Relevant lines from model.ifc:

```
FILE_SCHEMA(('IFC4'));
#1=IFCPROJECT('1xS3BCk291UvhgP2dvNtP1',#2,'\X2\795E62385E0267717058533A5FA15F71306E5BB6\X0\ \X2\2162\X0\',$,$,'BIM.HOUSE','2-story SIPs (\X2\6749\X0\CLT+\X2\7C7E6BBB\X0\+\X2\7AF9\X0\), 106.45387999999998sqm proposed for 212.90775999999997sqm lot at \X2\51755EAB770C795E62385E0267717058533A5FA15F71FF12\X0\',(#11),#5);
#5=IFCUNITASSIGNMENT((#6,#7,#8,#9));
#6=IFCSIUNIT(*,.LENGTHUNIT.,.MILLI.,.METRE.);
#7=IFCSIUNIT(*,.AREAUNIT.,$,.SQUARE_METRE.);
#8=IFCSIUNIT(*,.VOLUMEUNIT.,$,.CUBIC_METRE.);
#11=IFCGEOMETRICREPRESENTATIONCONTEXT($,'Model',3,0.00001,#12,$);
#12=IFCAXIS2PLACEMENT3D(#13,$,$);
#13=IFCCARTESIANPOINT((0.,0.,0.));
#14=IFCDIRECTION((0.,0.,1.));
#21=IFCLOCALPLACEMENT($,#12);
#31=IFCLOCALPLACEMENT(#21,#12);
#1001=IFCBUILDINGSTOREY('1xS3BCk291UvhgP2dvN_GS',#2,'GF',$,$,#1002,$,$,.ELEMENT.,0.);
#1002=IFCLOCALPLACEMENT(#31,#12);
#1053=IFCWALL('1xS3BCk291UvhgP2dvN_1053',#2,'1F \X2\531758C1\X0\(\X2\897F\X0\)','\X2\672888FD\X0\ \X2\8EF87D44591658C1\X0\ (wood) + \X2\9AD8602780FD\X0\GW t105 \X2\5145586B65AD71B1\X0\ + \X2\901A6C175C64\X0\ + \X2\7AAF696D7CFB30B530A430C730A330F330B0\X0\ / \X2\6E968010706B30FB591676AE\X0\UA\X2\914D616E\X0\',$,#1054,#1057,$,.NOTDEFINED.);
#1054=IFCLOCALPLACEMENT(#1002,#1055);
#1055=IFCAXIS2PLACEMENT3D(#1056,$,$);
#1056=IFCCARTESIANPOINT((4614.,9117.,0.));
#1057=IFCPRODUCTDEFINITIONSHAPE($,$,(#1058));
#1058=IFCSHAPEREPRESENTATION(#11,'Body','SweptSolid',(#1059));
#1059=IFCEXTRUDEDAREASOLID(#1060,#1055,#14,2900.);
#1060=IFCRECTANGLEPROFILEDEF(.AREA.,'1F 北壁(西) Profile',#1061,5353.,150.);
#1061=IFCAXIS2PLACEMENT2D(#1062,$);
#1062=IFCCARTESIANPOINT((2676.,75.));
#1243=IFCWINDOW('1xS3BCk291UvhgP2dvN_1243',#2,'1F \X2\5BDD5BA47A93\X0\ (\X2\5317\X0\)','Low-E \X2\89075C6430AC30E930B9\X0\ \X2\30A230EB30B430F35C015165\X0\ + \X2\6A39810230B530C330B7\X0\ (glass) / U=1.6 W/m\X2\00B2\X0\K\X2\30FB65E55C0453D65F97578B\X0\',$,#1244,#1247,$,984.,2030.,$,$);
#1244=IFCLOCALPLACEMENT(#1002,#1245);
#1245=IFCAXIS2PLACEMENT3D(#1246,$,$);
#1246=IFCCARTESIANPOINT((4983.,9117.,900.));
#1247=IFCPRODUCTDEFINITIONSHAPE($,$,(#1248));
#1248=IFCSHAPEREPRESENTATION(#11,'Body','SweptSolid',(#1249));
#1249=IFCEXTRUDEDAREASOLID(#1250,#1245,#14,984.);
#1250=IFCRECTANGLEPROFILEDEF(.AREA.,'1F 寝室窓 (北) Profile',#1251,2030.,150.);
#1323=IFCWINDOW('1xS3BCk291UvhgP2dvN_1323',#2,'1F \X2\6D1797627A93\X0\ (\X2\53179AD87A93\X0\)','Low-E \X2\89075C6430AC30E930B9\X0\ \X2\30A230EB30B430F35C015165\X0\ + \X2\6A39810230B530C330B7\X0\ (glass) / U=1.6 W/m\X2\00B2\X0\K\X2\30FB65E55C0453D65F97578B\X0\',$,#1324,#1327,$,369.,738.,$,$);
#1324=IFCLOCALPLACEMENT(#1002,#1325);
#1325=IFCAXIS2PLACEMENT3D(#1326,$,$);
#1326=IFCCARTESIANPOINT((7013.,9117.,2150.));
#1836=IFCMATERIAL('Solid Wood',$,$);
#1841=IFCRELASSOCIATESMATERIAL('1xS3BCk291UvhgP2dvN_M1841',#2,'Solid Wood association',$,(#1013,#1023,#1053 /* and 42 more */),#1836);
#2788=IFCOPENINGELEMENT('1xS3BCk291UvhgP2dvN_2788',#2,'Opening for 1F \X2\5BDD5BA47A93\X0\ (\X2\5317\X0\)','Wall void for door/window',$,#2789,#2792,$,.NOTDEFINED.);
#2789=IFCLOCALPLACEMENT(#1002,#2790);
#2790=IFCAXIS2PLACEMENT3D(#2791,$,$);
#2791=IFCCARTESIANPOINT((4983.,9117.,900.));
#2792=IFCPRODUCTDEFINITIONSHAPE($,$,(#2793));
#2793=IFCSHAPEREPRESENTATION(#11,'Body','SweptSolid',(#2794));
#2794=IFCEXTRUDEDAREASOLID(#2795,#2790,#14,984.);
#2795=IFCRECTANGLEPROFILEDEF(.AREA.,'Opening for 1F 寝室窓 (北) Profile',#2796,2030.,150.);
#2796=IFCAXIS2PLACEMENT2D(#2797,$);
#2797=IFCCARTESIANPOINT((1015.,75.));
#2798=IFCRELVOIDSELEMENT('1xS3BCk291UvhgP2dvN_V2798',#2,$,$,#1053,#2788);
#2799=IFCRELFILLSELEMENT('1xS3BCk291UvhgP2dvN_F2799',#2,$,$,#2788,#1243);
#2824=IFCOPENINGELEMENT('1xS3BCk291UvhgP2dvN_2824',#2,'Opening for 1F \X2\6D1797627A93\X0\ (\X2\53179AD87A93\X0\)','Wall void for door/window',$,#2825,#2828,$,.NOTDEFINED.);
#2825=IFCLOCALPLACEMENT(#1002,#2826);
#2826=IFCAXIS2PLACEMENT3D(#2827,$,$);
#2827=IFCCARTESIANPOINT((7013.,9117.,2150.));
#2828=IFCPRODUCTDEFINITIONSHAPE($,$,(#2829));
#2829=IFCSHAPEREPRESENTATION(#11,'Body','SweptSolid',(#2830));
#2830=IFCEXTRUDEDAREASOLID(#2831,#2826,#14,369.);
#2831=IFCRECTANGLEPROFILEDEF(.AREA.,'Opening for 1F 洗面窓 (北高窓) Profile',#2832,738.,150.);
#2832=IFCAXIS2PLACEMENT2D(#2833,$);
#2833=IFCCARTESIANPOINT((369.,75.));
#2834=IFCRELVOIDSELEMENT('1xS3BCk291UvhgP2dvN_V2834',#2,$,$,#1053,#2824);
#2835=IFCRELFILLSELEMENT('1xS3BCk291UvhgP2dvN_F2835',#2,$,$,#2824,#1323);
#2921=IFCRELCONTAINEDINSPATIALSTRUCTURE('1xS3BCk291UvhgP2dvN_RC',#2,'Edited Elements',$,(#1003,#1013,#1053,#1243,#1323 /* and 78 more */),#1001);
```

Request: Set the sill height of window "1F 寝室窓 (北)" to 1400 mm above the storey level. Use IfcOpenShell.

```python
import numpy as np
import ifcopenshell
import ifcopenshell.api.geometry
import ifcopenshell.geom
import ifcopenshell.util.element
import ifcopenshell.util.placement
import ifcopenshell.util.shape
import ifcopenshell.util.unit

model = ifcopenshell.open("model.ifc")
unit_scale = ifcopenshell.util.unit.calculate_unit_scale(model)

window = model.by_guid("1xS3BCk291UvhgP2dvN_1243")
opening = window.FillsVoids[0].RelatingOpeningElement
storey = ifcopenshell.util.element.get_container(window, ifc_class="IfcBuildingStorey")
level = ifcopenshell.util.placement.get_local_placement(storey.ObjectPlacement)[2, 3]

# The opening's origin need not be at the sill, so measure its lowest point.
shape = ifcopenshell.geom.create_shape(ifcopenshell.geom.settings(), opening)
bottom = ifcopenshell.util.shape.get_shape_bottom_elevation(shape, shape.geometry) / unit_scale
dz = level + 1400.0 - bottom

shift = np.array([0.0, 0.0, dz])
# The window is not placed relative to its opening, so move both.
for product in (opening, window):
    matrix = ifcopenshell.util.placement.get_local_placement(product.ObjectPlacement)
    matrix[:3, 3] += shift
    ifcopenshell.api.geometry.edit_object_placement(model, product=product, matrix=matrix, is_si=False)

print(f"moved by {dz * unit_scale:+.3f} m")

model.write("model_updated.ifc")
```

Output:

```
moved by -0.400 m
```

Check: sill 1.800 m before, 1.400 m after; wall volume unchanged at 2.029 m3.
